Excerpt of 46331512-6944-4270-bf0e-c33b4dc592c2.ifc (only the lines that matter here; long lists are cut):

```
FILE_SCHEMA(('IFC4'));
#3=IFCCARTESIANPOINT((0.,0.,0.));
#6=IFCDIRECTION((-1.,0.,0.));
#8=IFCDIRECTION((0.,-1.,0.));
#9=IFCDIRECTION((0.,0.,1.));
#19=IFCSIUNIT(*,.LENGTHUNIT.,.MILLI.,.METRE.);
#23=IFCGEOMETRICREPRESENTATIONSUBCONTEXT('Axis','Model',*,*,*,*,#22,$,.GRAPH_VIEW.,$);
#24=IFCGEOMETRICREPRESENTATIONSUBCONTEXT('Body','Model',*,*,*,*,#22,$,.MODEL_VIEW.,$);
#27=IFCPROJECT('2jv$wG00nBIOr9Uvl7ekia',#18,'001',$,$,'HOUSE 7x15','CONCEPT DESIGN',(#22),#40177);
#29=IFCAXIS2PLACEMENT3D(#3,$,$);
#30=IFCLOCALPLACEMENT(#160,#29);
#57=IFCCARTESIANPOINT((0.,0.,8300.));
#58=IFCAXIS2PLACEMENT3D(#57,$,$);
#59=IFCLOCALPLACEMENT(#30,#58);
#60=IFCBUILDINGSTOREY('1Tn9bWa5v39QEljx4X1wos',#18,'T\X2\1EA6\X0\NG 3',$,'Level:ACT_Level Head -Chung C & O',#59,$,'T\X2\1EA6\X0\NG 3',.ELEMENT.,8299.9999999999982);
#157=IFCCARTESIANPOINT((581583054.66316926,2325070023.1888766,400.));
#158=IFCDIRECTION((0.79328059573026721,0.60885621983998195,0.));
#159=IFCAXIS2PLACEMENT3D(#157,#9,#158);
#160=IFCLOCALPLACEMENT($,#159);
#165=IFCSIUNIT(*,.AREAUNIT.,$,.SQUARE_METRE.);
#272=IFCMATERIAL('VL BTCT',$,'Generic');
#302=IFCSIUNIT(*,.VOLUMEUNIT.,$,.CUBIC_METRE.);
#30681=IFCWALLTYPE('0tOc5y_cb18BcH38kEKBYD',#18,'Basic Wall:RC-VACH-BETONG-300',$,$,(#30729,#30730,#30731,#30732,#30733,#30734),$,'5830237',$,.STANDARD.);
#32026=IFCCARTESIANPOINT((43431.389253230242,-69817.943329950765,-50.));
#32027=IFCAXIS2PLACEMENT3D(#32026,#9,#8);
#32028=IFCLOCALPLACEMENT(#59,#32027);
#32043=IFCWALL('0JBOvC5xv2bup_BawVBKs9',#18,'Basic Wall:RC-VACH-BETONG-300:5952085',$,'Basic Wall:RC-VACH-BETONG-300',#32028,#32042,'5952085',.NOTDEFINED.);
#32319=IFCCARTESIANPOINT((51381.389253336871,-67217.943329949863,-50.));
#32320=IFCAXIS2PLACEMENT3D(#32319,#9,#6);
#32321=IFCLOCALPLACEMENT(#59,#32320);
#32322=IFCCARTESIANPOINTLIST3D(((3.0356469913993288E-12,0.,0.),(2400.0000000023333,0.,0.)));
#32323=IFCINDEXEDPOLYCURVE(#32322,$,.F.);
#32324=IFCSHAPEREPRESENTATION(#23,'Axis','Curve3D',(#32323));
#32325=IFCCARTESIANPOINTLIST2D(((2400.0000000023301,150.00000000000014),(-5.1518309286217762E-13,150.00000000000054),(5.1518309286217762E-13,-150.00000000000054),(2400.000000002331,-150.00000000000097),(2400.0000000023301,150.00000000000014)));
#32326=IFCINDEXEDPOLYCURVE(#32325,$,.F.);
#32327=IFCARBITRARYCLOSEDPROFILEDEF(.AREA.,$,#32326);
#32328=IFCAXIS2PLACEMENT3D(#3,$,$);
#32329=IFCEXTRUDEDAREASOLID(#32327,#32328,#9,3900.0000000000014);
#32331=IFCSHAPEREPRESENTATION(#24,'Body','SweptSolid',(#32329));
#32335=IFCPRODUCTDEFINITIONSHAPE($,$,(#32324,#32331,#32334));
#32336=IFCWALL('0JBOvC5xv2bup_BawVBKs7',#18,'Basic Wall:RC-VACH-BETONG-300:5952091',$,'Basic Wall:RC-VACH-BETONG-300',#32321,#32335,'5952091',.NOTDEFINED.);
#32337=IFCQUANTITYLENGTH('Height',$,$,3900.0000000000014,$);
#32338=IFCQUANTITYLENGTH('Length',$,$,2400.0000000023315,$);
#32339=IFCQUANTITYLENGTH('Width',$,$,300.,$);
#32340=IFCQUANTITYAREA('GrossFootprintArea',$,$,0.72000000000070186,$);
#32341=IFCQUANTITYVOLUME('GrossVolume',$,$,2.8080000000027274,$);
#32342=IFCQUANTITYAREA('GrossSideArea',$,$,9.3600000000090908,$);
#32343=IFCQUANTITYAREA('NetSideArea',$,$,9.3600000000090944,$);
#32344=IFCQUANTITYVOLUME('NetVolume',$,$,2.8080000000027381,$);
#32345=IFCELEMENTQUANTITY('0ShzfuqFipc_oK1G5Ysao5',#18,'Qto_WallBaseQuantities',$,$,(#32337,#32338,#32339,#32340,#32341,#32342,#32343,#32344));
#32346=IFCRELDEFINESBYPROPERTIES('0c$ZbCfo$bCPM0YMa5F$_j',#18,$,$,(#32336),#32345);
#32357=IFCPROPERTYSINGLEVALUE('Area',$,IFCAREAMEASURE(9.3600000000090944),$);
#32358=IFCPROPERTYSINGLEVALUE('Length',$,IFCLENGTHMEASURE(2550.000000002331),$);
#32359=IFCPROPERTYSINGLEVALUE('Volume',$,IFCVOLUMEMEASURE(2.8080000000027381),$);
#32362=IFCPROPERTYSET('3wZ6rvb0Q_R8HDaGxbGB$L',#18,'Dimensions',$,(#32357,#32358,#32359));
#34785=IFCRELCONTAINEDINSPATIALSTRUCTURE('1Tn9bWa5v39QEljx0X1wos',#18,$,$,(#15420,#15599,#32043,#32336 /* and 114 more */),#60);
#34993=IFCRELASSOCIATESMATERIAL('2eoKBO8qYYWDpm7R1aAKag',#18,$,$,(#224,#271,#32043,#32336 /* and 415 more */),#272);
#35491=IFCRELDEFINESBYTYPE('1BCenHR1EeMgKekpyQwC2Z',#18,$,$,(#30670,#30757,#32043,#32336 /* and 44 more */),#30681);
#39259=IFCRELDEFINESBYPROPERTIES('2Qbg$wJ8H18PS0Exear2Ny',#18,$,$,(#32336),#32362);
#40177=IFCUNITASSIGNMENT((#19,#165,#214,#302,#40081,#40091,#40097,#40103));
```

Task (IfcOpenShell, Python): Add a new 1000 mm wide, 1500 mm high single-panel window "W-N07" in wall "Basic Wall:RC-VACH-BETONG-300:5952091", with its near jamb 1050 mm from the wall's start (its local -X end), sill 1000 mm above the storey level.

```python
import numpy as np
import ifcopenshell
import ifcopenshell.api.feature
import ifcopenshell.api.geometry
import ifcopenshell.api.pset
import ifcopenshell.api.root
import ifcopenshell.api.spatial
import ifcopenshell.geom
import ifcopenshell.util.element
import ifcopenshell.util.placement
import ifcopenshell.util.representation
import ifcopenshell.util.shape
import ifcopenshell.util.unit

model = ifcopenshell.open("46331512-6944-4270-bf0e-c33b4dc592c2.ifc")
unit_scale = ifcopenshell.util.unit.calculate_unit_scale(model)
area_scale = ifcopenshell.util.unit.calculate_unit_scale(model, "AREAUNIT")
volume_scale = ifcopenshell.util.unit.calculate_unit_scale(model, "VOLUMEUNIT")
settings = ifcopenshell.geom.settings()


def volume(element):
    """Net volume in cubic metres, openings subtracted."""
    shape = ifcopenshell.geom.create_shape(settings, element)
    return ifcopenshell.util.shape.get_volume(shape.geometry)


wall = model.by_guid("0JBOvC5xv2bup_BawVBKs7")
storey = ifcopenshell.util.element.get_container(wall, ifc_class="IfcBuildingStorey")
context = ifcopenshell.util.representation.get_context(model, "Model", "Body", "MODEL_VIEW")
before = volume(wall)

width, height, from_end, sill = 1, 1.5, 1.05, 1  # metres

# The wall runs along its own X axis, and the end named is its -X end.
wall_shape = ifcopenshell.geom.create_shape(settings, wall)
x, y, z = ifcopenshell.util.shape.get_vertices(wall_shape.geometry).T
start = x.min() + from_end
face, thickness = float(y.min()), float(y.max() - y.min())
wall_matrix = ifcopenshell.util.placement.get_local_placement(wall.ObjectPlacement)
level = ifcopenshell.util.placement.get_local_placement(storey.ObjectPlacement)[2, 3]


def in_wall(x, y):
    """Placement at x, y metres in the wall's axes, at sill height."""
    matrix = wall_matrix.copy()
    matrix[:, 3] = wall_matrix @ np.array([x / unit_scale, y / unit_scale, 0.0, 1.0])
    matrix[2, 3] = level + sill / unit_scale
    return matrix


# Opening: a box that overshoots both wall faces by 50 mm.
opening = ifcopenshell.api.root.create_entity(model, ifc_class="IfcOpeningElement", predefined_type="OPENING")
box = ifcopenshell.api.geometry.add_wall_representation(
    model, context=context, length=width, height=height, thickness=thickness + 0.1
)
ifcopenshell.api.geometry.assign_representation(model, product=opening, representation=box)
ifcopenshell.api.geometry.edit_object_placement(model, product=opening, matrix=in_wall(start, face - 0.05), is_si=False)
ifcopenshell.api.feature.add_feature(model, feature=opening, element=wall)

window = ifcopenshell.api.root.create_entity(model, ifc_class="IfcWindow", name="W-N07", predefined_type="WINDOW")
window.OverallWidth, window.OverallHeight = width / unit_scale, height / unit_scale
window.PartitioningType = "SINGLE_PANEL"
body = ifcopenshell.api.geometry.add_window_representation(
    model,
    context=context,
    overall_width=window.OverallWidth,
    overall_height=window.OverallHeight,
    partition_type="SINGLE_PANEL",
)
ifcopenshell.api.geometry.assign_representation(model, product=window, representation=body)
ifcopenshell.api.spatial.assign_container(model, products=[window], relating_structure=storey)
ifcopenshell.api.feature.add_filling(model, opening=opening, element=window)

# Centre the window in the wall's thickness.
ifcopenshell.api.geometry.edit_object_placement(model, product=window, matrix=in_wall(start, face), is_si=False)
window_shape = ifcopenshell.geom.create_shape(settings, window)
depth = ifcopenshell.util.shape.get_vertices(window_shape.geometry)[:, 1]
offset = face + thickness / 2 - (depth.min() + depth.max()) / 2
ifcopenshell.api.geometry.edit_object_placement(model, product=window, matrix=in_wall(start, offset), is_si=False)

after = volume(wall)

# Update the wall's stored quantities.
qto = model.by_id(ifcopenshell.util.element.get_pset(wall, "Qto_WallBaseQuantities", should_inherit=False)["id"])
ifcopenshell.api.pset.edit_qto(model, qto=qto, properties={
    "NetSideArea": after / thickness / area_scale,
    "NetVolume": after / volume_scale,
})
pset = model.by_id(ifcopenshell.util.element.get_pset(wall, "Dimensions", should_inherit=False)["id"])
ifcopenshell.api.pset.edit_pset(model, pset=pset, properties={
    "Area": model.create_entity("IfcAreaMeasure", after / thickness / area_scale),
    "Volume": model.create_entity("IfcVolumeMeasure", after / volume_scale),
})

print(f"wall volume {before:.3f} -> {after:.3f} m3")

model.write("46331512-6944-4270-bf0e-c33b4dc592c2_updated.ifc")
```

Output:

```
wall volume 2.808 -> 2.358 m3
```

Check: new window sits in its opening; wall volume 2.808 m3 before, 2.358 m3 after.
